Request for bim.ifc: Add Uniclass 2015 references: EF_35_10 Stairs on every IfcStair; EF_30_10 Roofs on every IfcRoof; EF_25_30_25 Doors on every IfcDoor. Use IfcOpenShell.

First a look at what the model holds.

```python
import ifcopenshell

model = ifcopenshell.open("bim.ifc")
print(model.schema)
print("classifications:", [c.Name for c in model.by_type("IfcClassification")])
for ifc_class in ("IfcDoor", "IfcRoof", "IfcStair", "IfcWall", "IfcWindow"):
    print(ifc_class, len(model.by_type(ifc_class)))
```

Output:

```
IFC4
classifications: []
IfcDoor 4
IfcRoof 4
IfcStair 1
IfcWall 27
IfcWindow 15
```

```python
import ifcopenshell
import ifcopenshell.api.classification

model = ifcopenshell.open("bim.ifc")

system = ifcopenshell.api.classification.add_classification(model, classification="Uniclass 2015")

codes = {
    "IfcStair": ("EF_35_10", "Stairs"),
    "IfcRoof": ("EF_30_10", "Roofs"),
    "IfcDoor": ("EF_25_30_25", "Doors"),
}
for ifc_class, (code, name) in codes.items():
    products = model.by_type(ifc_class)
    ifcopenshell.api.classification.add_reference(
        model, products=products, classification=system, identification=code, name=name
    )
    print(code, len(products))

model.write("bim_updated.ifc")
```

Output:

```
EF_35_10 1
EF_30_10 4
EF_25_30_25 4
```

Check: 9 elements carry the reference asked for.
